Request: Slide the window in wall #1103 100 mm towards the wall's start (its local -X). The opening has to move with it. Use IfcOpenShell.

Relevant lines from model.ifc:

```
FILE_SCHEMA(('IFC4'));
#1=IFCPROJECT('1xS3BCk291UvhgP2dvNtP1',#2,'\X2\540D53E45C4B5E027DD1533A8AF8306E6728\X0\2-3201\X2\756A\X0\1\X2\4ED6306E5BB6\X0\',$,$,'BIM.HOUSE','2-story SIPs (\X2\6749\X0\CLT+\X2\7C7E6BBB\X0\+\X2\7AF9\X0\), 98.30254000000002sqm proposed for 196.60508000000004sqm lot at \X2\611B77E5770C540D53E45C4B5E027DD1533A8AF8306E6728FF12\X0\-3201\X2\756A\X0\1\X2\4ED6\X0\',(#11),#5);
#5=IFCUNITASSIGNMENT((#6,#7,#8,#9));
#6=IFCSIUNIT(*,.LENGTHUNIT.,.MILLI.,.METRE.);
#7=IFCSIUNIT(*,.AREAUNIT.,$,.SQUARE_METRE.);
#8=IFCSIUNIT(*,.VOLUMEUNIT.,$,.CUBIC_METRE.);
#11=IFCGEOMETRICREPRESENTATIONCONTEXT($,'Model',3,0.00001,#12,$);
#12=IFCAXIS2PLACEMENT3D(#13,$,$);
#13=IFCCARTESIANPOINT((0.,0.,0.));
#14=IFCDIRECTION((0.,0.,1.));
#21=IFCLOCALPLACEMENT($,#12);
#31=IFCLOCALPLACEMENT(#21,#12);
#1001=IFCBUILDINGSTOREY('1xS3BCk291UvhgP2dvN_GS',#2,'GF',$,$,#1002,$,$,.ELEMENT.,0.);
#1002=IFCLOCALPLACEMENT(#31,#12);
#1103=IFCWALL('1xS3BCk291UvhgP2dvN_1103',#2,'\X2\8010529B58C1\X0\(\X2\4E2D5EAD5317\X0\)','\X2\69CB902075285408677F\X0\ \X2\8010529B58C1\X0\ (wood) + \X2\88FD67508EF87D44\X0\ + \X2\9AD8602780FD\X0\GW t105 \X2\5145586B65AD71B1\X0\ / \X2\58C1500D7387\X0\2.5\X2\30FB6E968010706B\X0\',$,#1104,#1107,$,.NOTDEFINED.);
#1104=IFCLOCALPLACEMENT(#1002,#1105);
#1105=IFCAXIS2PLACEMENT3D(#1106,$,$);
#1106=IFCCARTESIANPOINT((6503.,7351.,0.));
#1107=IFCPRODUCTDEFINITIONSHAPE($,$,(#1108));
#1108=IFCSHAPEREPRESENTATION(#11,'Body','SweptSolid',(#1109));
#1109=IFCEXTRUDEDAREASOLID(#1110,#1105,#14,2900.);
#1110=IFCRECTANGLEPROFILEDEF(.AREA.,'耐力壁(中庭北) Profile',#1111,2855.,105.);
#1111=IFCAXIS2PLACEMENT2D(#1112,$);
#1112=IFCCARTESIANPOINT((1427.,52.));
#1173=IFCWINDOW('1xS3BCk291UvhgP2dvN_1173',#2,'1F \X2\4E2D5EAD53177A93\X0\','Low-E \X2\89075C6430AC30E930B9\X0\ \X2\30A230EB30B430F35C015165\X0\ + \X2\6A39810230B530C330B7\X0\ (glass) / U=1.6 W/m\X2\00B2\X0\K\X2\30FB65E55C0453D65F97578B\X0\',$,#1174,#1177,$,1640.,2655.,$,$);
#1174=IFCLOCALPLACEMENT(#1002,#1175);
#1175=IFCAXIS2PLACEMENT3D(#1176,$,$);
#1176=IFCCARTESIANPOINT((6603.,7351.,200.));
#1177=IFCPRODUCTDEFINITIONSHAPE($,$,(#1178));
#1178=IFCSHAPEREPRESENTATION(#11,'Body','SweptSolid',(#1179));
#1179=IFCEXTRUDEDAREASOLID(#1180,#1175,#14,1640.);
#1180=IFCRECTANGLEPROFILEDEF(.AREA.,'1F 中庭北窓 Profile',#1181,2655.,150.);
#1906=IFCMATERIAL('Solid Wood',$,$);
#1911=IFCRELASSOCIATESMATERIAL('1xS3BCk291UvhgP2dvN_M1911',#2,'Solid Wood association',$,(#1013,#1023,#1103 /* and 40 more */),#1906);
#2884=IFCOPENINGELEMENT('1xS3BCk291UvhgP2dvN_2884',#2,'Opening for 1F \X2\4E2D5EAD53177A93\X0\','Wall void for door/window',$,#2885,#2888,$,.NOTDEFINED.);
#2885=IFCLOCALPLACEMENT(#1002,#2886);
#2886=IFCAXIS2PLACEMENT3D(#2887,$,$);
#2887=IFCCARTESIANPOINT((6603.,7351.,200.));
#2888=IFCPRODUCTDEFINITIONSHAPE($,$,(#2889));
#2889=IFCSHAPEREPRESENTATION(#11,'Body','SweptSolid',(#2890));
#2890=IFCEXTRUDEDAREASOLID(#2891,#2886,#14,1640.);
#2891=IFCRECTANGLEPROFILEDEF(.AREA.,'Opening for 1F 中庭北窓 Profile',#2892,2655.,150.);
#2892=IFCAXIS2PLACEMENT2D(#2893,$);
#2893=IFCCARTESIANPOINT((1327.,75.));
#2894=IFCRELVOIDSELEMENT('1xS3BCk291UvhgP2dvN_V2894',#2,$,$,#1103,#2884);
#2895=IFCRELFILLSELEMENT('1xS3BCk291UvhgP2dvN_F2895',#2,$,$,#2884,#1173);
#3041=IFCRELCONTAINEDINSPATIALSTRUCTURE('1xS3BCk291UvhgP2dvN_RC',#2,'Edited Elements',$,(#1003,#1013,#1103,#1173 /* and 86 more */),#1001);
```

```python
import ifcopenshell
import ifcopenshell.api.geometry
import ifcopenshell.util.placement
import ifcopenshell.util.unit

model = ifcopenshell.open("model.ifc")
unit_scale = ifcopenshell.util.unit.calculate_unit_scale(model)

window = model.by_id(1173)
opening = window.FillsVoids[0].RelatingOpeningElement
wall = opening.VoidsElements[0].RelatingBuildingElement

wall_matrix = ifcopenshell.util.placement.get_local_placement(wall.ObjectPlacement)
shift = wall_matrix[:3, 0] * -0.1 / unit_scale
before = ifcopenshell.util.placement.get_local_placement(window.ObjectPlacement)[:3, 3].copy()

# The window is not placed relative to its opening, so move both.
for product in (opening, window):
    matrix = ifcopenshell.util.placement.get_local_placement(product.ObjectPlacement)
    matrix[:3, 3] += shift
    ifcopenshell.api.geometry.edit_object_placement(model, product=product, matrix=matrix, is_si=False)

after = ifcopenshell.util.placement.get_local_placement(window.ObjectPlacement)[:3, 3]
print("window moved by", (after - before).round(3) + 0.0)

model.write("model_v2.ifc")
```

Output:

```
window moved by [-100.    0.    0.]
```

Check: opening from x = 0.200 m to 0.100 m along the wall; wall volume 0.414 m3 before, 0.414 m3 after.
